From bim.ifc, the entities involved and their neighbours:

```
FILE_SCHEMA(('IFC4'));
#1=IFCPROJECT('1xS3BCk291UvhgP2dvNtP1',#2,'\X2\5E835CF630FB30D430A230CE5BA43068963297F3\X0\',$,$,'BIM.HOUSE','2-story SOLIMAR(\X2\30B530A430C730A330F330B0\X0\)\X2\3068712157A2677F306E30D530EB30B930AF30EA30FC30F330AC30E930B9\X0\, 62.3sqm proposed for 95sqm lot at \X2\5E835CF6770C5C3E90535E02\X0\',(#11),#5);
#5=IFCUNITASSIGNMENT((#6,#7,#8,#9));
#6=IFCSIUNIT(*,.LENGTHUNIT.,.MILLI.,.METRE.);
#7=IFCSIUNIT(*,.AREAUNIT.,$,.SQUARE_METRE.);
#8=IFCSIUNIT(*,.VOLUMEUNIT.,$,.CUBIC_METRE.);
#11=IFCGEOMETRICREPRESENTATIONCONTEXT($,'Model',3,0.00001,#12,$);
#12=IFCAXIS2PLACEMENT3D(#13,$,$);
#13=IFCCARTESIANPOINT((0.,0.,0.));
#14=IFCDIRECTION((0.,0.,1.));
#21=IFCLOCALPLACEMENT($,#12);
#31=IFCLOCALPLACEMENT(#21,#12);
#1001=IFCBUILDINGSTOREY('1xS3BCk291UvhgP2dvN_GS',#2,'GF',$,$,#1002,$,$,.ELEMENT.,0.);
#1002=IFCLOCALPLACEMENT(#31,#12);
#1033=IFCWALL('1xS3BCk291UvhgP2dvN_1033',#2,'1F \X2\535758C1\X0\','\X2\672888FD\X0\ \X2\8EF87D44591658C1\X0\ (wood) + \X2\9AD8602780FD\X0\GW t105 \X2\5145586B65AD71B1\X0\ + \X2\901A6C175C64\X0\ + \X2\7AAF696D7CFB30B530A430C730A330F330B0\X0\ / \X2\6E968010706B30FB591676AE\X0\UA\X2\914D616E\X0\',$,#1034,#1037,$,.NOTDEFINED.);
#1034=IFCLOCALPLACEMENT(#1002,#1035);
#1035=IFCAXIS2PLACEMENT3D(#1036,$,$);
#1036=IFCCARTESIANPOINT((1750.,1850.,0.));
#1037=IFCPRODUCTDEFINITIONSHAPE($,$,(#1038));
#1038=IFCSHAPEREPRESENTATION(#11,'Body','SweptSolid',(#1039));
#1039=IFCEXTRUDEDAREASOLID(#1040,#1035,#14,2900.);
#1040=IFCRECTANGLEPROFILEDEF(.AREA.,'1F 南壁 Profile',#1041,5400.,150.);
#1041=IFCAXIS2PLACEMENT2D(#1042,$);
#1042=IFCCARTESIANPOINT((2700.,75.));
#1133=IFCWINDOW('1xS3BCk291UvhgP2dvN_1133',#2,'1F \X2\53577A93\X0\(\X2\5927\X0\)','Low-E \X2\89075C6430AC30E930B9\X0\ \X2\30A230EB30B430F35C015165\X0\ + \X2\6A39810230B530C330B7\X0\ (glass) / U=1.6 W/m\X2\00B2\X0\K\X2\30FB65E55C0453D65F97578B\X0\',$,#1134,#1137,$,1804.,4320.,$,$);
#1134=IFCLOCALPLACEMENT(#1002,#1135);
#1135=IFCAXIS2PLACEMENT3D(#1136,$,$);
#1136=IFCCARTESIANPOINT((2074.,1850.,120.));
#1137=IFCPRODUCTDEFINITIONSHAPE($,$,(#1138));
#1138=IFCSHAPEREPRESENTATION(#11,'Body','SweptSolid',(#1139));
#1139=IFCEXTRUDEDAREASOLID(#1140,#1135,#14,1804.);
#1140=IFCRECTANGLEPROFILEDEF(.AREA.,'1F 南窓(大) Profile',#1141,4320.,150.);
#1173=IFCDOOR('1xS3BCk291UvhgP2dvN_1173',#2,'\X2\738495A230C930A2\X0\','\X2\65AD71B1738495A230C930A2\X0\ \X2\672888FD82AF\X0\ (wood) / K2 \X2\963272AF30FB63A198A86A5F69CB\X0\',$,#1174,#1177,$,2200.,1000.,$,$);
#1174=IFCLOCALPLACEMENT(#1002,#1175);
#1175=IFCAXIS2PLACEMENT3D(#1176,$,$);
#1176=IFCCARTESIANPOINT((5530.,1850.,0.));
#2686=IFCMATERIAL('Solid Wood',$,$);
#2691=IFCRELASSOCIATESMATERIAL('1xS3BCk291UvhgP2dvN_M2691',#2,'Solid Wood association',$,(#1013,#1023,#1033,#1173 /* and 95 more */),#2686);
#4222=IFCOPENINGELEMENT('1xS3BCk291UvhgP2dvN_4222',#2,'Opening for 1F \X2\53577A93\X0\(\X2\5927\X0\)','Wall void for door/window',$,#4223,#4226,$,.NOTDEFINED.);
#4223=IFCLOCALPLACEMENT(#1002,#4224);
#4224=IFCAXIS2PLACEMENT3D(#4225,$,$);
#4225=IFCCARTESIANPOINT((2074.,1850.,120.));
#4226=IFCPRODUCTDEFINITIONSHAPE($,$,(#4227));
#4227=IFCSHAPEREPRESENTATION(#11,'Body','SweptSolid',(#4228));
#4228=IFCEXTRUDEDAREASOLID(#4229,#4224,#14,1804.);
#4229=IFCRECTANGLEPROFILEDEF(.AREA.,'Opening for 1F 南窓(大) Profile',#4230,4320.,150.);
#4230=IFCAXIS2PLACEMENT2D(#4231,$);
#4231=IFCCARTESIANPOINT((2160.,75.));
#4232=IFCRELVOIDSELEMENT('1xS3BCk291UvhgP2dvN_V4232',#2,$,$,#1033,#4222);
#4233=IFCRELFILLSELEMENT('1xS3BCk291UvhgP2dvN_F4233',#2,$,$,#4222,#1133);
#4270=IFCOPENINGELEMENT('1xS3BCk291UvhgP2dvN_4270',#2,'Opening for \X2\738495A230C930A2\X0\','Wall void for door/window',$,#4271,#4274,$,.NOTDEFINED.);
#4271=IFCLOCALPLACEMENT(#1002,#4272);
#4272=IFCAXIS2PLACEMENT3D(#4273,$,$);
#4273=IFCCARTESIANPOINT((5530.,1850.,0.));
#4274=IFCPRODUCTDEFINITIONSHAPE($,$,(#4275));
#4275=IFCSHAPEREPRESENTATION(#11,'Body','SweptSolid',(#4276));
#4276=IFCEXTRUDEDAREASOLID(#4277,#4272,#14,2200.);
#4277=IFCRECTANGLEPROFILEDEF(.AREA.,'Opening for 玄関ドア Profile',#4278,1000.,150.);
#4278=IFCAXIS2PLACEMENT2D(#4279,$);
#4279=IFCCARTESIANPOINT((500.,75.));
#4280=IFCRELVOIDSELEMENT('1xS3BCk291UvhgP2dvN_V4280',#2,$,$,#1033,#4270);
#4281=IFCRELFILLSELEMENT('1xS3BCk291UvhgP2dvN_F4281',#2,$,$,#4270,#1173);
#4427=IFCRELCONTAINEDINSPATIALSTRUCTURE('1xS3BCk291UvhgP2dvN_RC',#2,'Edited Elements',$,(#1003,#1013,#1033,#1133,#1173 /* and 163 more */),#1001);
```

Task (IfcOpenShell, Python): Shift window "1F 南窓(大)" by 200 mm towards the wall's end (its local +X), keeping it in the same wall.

```python
import ifcopenshell
import ifcopenshell.api.geometry
import ifcopenshell.util.placement
import ifcopenshell.util.unit

model = ifcopenshell.open("bim.ifc")
unit_scale = ifcopenshell.util.unit.calculate_unit_scale(model)

window = model.by_guid("1xS3BCk291UvhgP2dvN_1133")
opening = window.FillsVoids[0].RelatingOpeningElement
wall = opening.VoidsElements[0].RelatingBuildingElement

wall_matrix = ifcopenshell.util.placement.get_local_placement(wall.ObjectPlacement)
shift = wall_matrix[:3, 0] * 0.2 / unit_scale
before = ifcopenshell.util.placement.get_local_placement(window.ObjectPlacement)[:3, 3].copy()

# The window is not placed relative to its opening, so move both.
for product in (opening, window):
    matrix = ifcopenshell.util.placement.get_local_placement(product.ObjectPlacement)
    matrix[:3, 3] += shift
    ifcopenshell.api.geometry.edit_object_placement(model, product=product, matrix=matrix, is_si=False)

after = ifcopenshell.util.placement.get_local_placement(window.ObjectPlacement)[:3, 3]
print("window moved by", (after - before).round(3) + 0.0)

model.write("bim_rev.ifc")
```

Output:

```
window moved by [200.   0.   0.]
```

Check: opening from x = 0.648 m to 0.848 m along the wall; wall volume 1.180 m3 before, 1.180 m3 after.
